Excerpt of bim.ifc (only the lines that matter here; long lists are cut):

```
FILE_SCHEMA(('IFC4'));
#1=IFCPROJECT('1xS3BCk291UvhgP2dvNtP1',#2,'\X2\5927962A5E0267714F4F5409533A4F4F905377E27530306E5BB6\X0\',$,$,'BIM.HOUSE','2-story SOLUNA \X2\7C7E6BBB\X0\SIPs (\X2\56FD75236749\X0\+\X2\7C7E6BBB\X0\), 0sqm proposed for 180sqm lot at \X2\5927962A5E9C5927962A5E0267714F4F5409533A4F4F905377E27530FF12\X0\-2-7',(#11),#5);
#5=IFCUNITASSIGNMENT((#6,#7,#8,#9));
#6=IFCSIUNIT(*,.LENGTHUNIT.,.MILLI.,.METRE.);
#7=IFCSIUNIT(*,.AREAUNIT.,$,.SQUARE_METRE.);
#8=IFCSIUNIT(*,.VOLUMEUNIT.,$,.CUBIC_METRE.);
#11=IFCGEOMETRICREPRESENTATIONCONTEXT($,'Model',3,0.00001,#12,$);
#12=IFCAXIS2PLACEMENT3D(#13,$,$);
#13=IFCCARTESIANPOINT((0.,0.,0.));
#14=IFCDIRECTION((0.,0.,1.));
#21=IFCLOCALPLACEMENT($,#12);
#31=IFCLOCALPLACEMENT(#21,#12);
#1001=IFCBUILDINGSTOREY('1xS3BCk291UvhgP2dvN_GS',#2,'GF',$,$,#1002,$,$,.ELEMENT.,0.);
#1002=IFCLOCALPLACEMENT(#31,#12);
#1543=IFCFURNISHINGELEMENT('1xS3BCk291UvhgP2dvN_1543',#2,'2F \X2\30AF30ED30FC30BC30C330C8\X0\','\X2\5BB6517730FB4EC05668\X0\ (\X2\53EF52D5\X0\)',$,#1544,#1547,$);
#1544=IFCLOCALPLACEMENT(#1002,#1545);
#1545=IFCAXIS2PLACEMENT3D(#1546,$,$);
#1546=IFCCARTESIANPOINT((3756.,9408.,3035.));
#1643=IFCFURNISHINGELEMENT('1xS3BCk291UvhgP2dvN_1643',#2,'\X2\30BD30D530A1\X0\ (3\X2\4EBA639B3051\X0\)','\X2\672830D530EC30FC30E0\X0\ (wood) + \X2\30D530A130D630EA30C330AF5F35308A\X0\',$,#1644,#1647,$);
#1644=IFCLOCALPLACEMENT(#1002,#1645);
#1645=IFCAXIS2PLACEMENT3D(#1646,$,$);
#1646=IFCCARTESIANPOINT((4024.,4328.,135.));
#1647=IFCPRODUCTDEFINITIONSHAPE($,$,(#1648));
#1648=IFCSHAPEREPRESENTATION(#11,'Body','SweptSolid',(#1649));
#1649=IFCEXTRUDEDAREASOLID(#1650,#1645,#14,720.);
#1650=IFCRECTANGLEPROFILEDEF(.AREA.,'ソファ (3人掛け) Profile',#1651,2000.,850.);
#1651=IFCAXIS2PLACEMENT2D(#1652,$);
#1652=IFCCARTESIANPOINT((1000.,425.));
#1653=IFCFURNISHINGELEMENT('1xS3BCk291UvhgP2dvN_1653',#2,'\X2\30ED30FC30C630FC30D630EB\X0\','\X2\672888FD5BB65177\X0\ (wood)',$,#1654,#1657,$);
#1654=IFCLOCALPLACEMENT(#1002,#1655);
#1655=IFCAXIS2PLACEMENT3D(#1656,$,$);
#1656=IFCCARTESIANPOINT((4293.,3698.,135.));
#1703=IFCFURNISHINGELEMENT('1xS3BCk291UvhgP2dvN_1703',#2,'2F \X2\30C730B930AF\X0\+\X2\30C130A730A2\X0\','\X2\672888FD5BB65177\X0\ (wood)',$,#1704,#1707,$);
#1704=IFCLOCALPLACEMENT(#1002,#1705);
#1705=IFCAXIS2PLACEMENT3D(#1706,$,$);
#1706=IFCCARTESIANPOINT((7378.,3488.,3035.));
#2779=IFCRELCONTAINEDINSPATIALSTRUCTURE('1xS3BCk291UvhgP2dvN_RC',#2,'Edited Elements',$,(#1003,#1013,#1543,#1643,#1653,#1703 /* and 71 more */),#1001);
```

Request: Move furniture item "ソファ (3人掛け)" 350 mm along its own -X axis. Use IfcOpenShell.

```python
import ifcopenshell
import ifcopenshell.api.geometry
import ifcopenshell.util.placement

model = ifcopenshell.open("bim.ifc")

item = model.by_guid("1xS3BCk291UvhgP2dvN_1643")
matrix = ifcopenshell.util.placement.get_local_placement(item.ObjectPlacement)
matrix[:3, 3] -= matrix[:3, 0] * 350.0
ifcopenshell.api.geometry.edit_object_placement(model, product=item, matrix=matrix, is_si=False)

print(ifcopenshell.util.placement.get_local_placement(item.ObjectPlacement).round(3) + 0.0)

model.write("bim_rev.ifc")
```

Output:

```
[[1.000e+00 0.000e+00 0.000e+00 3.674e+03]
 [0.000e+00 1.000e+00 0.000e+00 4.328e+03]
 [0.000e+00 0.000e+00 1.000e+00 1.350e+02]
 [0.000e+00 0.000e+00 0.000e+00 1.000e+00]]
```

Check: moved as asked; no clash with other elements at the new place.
